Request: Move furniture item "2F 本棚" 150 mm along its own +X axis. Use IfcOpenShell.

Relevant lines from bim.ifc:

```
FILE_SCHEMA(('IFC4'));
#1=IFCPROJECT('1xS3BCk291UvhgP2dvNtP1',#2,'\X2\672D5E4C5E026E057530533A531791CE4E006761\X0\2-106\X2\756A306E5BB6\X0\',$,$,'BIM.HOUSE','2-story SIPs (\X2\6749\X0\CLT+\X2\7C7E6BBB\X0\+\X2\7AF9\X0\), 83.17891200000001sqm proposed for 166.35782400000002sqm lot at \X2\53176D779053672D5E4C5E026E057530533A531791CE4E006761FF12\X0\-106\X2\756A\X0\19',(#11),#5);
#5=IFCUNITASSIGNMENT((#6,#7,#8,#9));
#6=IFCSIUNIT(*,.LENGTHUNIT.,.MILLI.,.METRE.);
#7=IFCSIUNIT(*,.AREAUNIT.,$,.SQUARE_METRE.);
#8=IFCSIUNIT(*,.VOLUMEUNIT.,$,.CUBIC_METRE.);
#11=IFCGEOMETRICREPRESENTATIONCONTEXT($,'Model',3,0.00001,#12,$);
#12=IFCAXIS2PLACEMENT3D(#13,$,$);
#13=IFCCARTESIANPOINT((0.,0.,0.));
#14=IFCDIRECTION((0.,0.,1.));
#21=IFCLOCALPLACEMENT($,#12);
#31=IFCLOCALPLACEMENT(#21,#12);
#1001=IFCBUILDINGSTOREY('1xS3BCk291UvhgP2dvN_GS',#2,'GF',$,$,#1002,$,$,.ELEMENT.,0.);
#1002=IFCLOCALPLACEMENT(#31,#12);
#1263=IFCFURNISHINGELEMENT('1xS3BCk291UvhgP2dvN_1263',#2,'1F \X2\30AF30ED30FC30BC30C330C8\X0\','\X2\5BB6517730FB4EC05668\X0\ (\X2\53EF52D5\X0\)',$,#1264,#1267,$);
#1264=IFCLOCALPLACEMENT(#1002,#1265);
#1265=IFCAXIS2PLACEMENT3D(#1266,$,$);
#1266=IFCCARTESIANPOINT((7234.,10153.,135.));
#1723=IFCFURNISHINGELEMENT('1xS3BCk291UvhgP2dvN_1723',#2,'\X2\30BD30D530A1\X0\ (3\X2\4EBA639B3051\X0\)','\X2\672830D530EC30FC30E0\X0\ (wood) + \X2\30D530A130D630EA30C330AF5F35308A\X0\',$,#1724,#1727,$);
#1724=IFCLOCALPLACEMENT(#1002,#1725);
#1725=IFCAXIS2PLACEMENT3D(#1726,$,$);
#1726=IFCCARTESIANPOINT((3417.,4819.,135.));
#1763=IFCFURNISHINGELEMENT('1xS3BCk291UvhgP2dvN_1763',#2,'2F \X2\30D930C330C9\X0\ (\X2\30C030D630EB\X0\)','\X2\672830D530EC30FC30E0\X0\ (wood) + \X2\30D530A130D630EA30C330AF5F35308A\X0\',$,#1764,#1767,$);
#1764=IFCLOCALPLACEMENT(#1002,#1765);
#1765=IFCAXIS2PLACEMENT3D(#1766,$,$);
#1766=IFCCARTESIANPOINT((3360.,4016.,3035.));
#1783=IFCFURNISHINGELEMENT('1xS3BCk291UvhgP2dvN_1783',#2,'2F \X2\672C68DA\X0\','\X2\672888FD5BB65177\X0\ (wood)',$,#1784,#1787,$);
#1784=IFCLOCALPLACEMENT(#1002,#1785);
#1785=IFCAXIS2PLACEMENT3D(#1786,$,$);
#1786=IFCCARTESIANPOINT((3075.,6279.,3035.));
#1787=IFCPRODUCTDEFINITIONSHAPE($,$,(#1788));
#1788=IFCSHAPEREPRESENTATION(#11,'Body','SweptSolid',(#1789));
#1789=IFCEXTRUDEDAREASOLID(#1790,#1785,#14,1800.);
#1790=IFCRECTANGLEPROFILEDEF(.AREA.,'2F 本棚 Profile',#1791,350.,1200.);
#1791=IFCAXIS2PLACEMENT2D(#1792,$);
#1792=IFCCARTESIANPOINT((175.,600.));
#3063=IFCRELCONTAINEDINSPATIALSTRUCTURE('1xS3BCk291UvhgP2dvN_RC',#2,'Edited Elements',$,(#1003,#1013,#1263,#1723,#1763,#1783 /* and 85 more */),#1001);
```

```python
import ifcopenshell
import ifcopenshell.api.geometry
import ifcopenshell.util.placement

model = ifcopenshell.open("bim.ifc")

item = model.by_id(1783)
matrix = ifcopenshell.util.placement.get_local_placement(item.ObjectPlacement)
matrix[:3, 3] += matrix[:3, 0] * 150.0
ifcopenshell.api.geometry.edit_object_placement(model, product=item, matrix=matrix, is_si=False)

print(ifcopenshell.util.placement.get_local_placement(item.ObjectPlacement).round(3) + 0.0)

model.write("bim_v2.ifc")
```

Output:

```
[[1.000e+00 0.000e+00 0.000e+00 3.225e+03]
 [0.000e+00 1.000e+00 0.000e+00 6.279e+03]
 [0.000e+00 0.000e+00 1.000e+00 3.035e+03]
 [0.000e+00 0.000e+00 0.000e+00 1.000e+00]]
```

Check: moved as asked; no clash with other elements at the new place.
